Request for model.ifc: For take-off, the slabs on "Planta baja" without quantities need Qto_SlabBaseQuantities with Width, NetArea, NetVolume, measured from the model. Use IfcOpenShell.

First a look at what the model holds.

```python
import ifcopenshell
import ifcopenshell.util.element
import ifcopenshell.util.unit

model = ifcopenshell.open("model.ifc")
print(model.schema)
for unit_type in ("LENGTHUNIT", "AREAUNIT", "VOLUMEUNIT"):
    print(unit_type, ifcopenshell.util.unit.calculate_unit_scale(model, unit_type))
storey = next(s for s in model.by_type("IfcBuildingStorey") if s.Name == "Planta baja")
slabs = [e for e in ifcopenshell.util.element.get_decomposition(storey) if e.is_a("IfcSlab")]
for e in sorted(slabs, key=lambda e: e.id()):
    print(e.id(), e.is_a(), e.Name, list(ifcopenshell.util.element.get_psets(e, qtos_only=True)), sep=" | ")
```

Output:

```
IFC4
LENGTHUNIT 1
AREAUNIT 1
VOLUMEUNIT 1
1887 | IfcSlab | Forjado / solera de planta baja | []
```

```python
import ifcopenshell
import ifcopenshell.api.pset
import ifcopenshell.geom
import ifcopenshell.util.element
import ifcopenshell.util.shape
import ifcopenshell.util.unit

model = ifcopenshell.open("model.ifc")
unit_scale = ifcopenshell.util.unit.calculate_unit_scale(model)
area_scale = ifcopenshell.util.unit.calculate_unit_scale(model, "AREAUNIT")
volume_scale = ifcopenshell.util.unit.calculate_unit_scale(model, "VOLUMEUNIT")
settings = ifcopenshell.geom.settings()

storey = next(s for s in model.by_type("IfcBuildingStorey") if s.Name == "Planta baja")
slabs = [e for e in ifcopenshell.util.element.get_decomposition(storey) if e.is_a("IfcSlab")]

for e in sorted(slabs, key=lambda e: e.id()):
    if ifcopenshell.util.element.get_psets(e, qtos_only=True, should_inherit=False):
        continue
    # Geometry comes back in metres, in the element's own axes.
    shape = ifcopenshell.geom.create_shape(settings, e)
    values = {
        "Width": ifcopenshell.util.shape.get_z(shape.geometry) / unit_scale,
        "NetArea": ifcopenshell.util.shape.get_footprint_area(shape.geometry) / area_scale,
        "NetVolume": ifcopenshell.util.shape.get_volume(shape.geometry) / volume_scale,
    }
    qto = ifcopenshell.api.pset.add_qto(model, product=e, name="Qto_SlabBaseQuantities")
    ifcopenshell.api.pset.edit_qto(model, qto=qto, properties=values)
    print(e.id(), {k: round(v, 3) for k, v in values.items()})

model.write("model_rev.ifc")
```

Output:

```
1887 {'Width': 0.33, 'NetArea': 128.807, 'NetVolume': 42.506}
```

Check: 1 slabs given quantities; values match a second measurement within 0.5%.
